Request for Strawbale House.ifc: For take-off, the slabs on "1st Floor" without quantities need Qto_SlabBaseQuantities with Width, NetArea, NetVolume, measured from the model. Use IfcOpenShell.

First a look at what the model holds.

```python
import ifcopenshell
import ifcopenshell.util.element
import ifcopenshell.util.unit

model = ifcopenshell.open("Strawbale House.ifc")
print(model.schema)
for unit_type in ("LENGTHUNIT", "AREAUNIT", "VOLUMEUNIT"):
    print(unit_type, ifcopenshell.util.unit.calculate_unit_scale(model, unit_type))
storey = next(s for s in model.by_type("IfcBuildingStorey") if s.Name == "1st Floor")
slabs = [e for e in ifcopenshell.util.element.get_decomposition(storey) if e.is_a("IfcSlab")]
for e in sorted(slabs, key=lambda e: e.id()):
    print(e.id(), e.is_a(), e.Name, list(ifcopenshell.util.element.get_psets(e, qtos_only=True)), sep=" | ")
```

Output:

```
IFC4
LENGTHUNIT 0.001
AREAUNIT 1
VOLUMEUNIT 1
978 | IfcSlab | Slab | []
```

```python
import ifcopenshell
import ifcopenshell.api.pset
import ifcopenshell.geom
import ifcopenshell.util.element
import ifcopenshell.util.shape
import ifcopenshell.util.unit

model = ifcopenshell.open("Strawbale House.ifc")
unit_scale = ifcopenshell.util.unit.calculate_unit_scale(model)
area_scale = ifcopenshell.util.unit.calculate_unit_scale(model, "AREAUNIT")
volume_scale = ifcopenshell.util.unit.calculate_unit_scale(model, "VOLUMEUNIT")
settings = ifcopenshell.geom.settings()

storey = next(s for s in model.by_type("IfcBuildingStorey") if s.Name == "1st Floor")
slabs = [e for e in ifcopenshell.util.element.get_decomposition(storey) if e.is_a("IfcSlab")]

for e in sorted(slabs, key=lambda e: e.id()):
    if ifcopenshell.util.element.get_psets(e, qtos_only=True, should_inherit=False):
        continue
    # Geometry comes back in metres, in the element's own axes.
    shape = ifcopenshell.geom.create_shape(settings, e)
    values = {
        "Width": ifcopenshell.util.shape.get_z(shape.geometry) / unit_scale,
        "NetArea": ifcopenshell.util.shape.get_footprint_area(shape.geometry) / area_scale,
        "NetVolume": ifcopenshell.util.shape.get_volume(shape.geometry) / volume_scale,
    }
    qto = ifcopenshell.api.pset.add_qto(model, product=e, name="Qto_SlabBaseQuantities")
    ifcopenshell.api.pset.edit_qto(model, qto=qto, properties=values)
    print(e.id(), {k: round(v, 3) for k, v in values.items()})

model.write("Strawbale House_v2.ifc")
```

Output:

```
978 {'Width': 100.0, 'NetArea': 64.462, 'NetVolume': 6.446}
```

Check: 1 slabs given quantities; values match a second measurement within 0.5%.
